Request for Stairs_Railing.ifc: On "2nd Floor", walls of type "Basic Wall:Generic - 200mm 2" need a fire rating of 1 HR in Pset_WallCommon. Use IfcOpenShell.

First a look at what the model holds.

```python
import ifcopenshell
import ifcopenshell.util.element

model = ifcopenshell.open("Stairs_Railing.ifc")
print(model.schema)
storey = next(s for s in model.by_type("IfcBuildingStorey") if s.Name == "2nd Floor")
walls = [e for e in ifcopenshell.util.element.get_decomposition(storey) if e.is_a("IfcWall")]
seen = {}
for e in walls:
    element_type = ifcopenshell.util.element.get_type(e)
    key = (element_type.Name if element_type != e and element_type else None, ifcopenshell.util.element.get_pset(e, "Pset_WallCommon", "FireRating"))
    seen[key] = seen.get(key, 0) + 1
for (name, value), count in sorted(seen.items(), key=str):
    print(count, "x", name, "|", value)
```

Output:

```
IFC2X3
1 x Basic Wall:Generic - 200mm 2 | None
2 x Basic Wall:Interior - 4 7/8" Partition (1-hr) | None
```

```python
import ifcopenshell
import ifcopenshell.api.pset
import ifcopenshell.util.element

model = ifcopenshell.open("Stairs_Railing.ifc")

storey = next(s for s in model.by_type("IfcBuildingStorey") if s.Name == "2nd Floor")
walls = [e for e in ifcopenshell.util.element.get_decomposition(storey) if e.is_a("IfcWall")]

count = 0
for e in walls:
    element_type = ifcopenshell.util.element.get_type(e)
    if element_type in (None, e) or element_type.Name != "Basic Wall:Generic - 200mm 2":
        continue
    # add_pset returns the element's existing set when there is one.
    pset = ifcopenshell.api.pset.add_pset(model, product=e, name="Pset_WallCommon")
    ifcopenshell.api.pset.edit_pset(model, pset=pset, properties={"FireRating": "1 HR"})
    count += 1

print(count, "walls updated")

model.write("Stairs_Railing_updated.ifc")
```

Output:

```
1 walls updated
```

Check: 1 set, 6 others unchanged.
